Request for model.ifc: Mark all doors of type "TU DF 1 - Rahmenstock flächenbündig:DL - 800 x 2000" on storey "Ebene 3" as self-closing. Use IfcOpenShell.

First a look at what the model holds.

```python
import ifcopenshell
import ifcopenshell.util.element

model = ifcopenshell.open("model.ifc")
print(model.schema)
storey = next(s for s in model.by_type("IfcBuildingStorey") if s.Name == "Ebene 3")
doors = [e for e in ifcopenshell.util.element.get_decomposition(storey) if e.is_a("IfcDoor")]
seen = {}
for e in doors:
    element_type = ifcopenshell.util.element.get_type(e)
    key = (element_type.Name if element_type != e and element_type else None, ifcopenshell.util.element.get_pset(e, "Pset_DoorCommon", "SelfClosing"))
    seen[key] = seen.get(key, 0) + 1
for (name, value), count in sorted(seen.items(), key=str):
    print(count, "x", name, "|", value)
```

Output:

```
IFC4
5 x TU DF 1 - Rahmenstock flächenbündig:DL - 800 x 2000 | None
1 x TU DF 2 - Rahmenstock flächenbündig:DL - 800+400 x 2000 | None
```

```python
import ifcopenshell
import ifcopenshell.api.pset
import ifcopenshell.util.element

model = ifcopenshell.open("model.ifc")

storey = next(s for s in model.by_type("IfcBuildingStorey") if s.Name == "Ebene 3")
doors = [e for e in ifcopenshell.util.element.get_decomposition(storey) if e.is_a("IfcDoor")]

count = 0
for e in doors:
    element_type = ifcopenshell.util.element.get_type(e)
    if element_type in (None, e) or element_type.Name != "TU DF 1 - Rahmenstock flächenbündig:DL - 800 x 2000":
        continue
    # add_pset returns the element's existing set when there is one.
    pset = ifcopenshell.api.pset.add_pset(model, product=e, name="Pset_DoorCommon")
    ifcopenshell.api.pset.edit_pset(model, pset=pset, properties={"SelfClosing": True})
    count += 1

print(count, "doors updated")

model.write("model_rev.ifc")
```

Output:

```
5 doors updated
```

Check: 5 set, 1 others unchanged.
